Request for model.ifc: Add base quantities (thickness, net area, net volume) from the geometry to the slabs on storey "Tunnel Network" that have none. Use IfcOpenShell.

First a look at what the model holds.

```python
import ifcopenshell
import ifcopenshell.util.element
import ifcopenshell.util.unit

model = ifcopenshell.open("model.ifc")
print(model.schema)
for unit_type in ("LENGTHUNIT", "AREAUNIT", "VOLUMEUNIT"):
    print(unit_type, ifcopenshell.util.unit.calculate_unit_scale(model, unit_type))
storey = next(s for s in model.by_type("IfcBuildingStorey") if s.Name == "Tunnel Network")
slabs = [e for e in ifcopenshell.util.element.get_decomposition(storey) if e.is_a("IfcSlab")]
for e in sorted(slabs, key=lambda e: e.id()):
    print(e.id(), e.is_a(), e.Name, list(ifcopenshell.util.element.get_psets(e, qtos_only=True)), sep=" | ")
```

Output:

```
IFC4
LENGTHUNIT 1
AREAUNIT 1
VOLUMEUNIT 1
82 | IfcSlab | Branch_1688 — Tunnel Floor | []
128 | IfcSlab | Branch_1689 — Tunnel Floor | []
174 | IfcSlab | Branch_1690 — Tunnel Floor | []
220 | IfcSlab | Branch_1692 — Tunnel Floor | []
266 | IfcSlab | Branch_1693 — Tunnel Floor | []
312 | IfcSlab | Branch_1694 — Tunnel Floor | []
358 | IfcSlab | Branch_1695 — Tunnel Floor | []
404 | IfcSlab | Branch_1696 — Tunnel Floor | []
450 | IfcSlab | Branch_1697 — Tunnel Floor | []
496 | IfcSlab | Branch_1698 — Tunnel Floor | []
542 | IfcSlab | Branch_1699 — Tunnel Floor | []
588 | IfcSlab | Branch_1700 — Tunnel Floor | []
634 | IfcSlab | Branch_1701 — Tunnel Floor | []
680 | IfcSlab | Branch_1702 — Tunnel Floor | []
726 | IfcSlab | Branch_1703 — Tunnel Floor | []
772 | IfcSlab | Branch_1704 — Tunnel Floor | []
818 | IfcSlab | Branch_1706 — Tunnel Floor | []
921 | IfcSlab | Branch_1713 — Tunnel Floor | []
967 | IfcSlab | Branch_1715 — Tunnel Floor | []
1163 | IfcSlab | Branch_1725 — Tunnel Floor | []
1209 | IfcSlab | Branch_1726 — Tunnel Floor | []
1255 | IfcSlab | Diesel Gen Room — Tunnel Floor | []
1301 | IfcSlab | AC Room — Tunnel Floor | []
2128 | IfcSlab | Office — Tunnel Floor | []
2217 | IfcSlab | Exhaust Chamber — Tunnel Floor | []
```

```python
import ifcopenshell
import ifcopenshell.api.pset
import ifcopenshell.geom
import ifcopenshell.util.element
import ifcopenshell.util.shape
import ifcopenshell.util.unit

model = ifcopenshell.open("model.ifc")
unit_scale = ifcopenshell.util.unit.calculate_unit_scale(model)
area_scale = ifcopenshell.util.unit.calculate_unit_scale(model, "AREAUNIT")
volume_scale = ifcopenshell.util.unit.calculate_unit_scale(model, "VOLUMEUNIT")
settings = ifcopenshell.geom.settings()

storey = next(s for s in model.by_type("IfcBuildingStorey") if s.Name == "Tunnel Network")
slabs = [e for e in ifcopenshell.util.element.get_decomposition(storey) if e.is_a("IfcSlab")]

for e in sorted(slabs, key=lambda e: e.id()):
    if ifcopenshell.util.element.get_psets(e, qtos_only=True, should_inherit=False):
        continue
    # Geometry comes back in metres, in the element's own axes.
    shape = ifcopenshell.geom.create_shape(settings, e)
    values = {
        "Width": ifcopenshell.util.shape.get_z(shape.geometry) / unit_scale,
        "NetArea": ifcopenshell.util.shape.get_footprint_area(shape.geometry) / area_scale,
        "NetVolume": ifcopenshell.util.shape.get_volume(shape.geometry) / volume_scale,
    }
    qto = ifcopenshell.api.pset.add_qto(model, product=e, name="Qto_SlabBaseQuantities")
    ifcopenshell.api.pset.edit_qto(model, qto=qto, properties=values)
    print(e.id(), {k: round(v, 3) for k, v in values.items()})

model.write("model_updated.ifc")
```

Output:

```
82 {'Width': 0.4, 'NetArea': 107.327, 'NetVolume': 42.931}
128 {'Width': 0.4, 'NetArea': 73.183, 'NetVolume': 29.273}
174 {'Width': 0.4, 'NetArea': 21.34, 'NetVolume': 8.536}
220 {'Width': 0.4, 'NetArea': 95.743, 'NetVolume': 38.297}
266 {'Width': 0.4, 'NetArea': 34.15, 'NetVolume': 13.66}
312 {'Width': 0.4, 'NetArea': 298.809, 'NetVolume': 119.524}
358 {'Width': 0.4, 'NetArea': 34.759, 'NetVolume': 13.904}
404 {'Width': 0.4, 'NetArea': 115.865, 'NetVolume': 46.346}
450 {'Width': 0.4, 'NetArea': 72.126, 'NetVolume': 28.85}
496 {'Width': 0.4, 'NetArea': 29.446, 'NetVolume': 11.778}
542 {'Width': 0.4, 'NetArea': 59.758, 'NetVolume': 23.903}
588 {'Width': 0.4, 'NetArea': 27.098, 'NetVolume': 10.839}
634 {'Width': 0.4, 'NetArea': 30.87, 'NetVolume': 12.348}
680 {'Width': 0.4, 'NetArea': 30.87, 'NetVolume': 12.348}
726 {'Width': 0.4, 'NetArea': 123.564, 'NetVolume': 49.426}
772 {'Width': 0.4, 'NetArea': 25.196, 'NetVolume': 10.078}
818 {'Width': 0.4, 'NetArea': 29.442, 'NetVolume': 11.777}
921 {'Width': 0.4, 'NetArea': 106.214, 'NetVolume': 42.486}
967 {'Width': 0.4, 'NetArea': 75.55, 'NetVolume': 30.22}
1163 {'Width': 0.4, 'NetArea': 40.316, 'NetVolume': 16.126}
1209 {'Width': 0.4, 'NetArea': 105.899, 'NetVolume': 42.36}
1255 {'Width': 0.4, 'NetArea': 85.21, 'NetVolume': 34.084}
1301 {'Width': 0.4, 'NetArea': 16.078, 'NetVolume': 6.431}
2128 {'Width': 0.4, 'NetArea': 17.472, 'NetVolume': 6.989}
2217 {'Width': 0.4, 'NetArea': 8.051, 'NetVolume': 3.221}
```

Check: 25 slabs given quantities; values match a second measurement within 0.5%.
